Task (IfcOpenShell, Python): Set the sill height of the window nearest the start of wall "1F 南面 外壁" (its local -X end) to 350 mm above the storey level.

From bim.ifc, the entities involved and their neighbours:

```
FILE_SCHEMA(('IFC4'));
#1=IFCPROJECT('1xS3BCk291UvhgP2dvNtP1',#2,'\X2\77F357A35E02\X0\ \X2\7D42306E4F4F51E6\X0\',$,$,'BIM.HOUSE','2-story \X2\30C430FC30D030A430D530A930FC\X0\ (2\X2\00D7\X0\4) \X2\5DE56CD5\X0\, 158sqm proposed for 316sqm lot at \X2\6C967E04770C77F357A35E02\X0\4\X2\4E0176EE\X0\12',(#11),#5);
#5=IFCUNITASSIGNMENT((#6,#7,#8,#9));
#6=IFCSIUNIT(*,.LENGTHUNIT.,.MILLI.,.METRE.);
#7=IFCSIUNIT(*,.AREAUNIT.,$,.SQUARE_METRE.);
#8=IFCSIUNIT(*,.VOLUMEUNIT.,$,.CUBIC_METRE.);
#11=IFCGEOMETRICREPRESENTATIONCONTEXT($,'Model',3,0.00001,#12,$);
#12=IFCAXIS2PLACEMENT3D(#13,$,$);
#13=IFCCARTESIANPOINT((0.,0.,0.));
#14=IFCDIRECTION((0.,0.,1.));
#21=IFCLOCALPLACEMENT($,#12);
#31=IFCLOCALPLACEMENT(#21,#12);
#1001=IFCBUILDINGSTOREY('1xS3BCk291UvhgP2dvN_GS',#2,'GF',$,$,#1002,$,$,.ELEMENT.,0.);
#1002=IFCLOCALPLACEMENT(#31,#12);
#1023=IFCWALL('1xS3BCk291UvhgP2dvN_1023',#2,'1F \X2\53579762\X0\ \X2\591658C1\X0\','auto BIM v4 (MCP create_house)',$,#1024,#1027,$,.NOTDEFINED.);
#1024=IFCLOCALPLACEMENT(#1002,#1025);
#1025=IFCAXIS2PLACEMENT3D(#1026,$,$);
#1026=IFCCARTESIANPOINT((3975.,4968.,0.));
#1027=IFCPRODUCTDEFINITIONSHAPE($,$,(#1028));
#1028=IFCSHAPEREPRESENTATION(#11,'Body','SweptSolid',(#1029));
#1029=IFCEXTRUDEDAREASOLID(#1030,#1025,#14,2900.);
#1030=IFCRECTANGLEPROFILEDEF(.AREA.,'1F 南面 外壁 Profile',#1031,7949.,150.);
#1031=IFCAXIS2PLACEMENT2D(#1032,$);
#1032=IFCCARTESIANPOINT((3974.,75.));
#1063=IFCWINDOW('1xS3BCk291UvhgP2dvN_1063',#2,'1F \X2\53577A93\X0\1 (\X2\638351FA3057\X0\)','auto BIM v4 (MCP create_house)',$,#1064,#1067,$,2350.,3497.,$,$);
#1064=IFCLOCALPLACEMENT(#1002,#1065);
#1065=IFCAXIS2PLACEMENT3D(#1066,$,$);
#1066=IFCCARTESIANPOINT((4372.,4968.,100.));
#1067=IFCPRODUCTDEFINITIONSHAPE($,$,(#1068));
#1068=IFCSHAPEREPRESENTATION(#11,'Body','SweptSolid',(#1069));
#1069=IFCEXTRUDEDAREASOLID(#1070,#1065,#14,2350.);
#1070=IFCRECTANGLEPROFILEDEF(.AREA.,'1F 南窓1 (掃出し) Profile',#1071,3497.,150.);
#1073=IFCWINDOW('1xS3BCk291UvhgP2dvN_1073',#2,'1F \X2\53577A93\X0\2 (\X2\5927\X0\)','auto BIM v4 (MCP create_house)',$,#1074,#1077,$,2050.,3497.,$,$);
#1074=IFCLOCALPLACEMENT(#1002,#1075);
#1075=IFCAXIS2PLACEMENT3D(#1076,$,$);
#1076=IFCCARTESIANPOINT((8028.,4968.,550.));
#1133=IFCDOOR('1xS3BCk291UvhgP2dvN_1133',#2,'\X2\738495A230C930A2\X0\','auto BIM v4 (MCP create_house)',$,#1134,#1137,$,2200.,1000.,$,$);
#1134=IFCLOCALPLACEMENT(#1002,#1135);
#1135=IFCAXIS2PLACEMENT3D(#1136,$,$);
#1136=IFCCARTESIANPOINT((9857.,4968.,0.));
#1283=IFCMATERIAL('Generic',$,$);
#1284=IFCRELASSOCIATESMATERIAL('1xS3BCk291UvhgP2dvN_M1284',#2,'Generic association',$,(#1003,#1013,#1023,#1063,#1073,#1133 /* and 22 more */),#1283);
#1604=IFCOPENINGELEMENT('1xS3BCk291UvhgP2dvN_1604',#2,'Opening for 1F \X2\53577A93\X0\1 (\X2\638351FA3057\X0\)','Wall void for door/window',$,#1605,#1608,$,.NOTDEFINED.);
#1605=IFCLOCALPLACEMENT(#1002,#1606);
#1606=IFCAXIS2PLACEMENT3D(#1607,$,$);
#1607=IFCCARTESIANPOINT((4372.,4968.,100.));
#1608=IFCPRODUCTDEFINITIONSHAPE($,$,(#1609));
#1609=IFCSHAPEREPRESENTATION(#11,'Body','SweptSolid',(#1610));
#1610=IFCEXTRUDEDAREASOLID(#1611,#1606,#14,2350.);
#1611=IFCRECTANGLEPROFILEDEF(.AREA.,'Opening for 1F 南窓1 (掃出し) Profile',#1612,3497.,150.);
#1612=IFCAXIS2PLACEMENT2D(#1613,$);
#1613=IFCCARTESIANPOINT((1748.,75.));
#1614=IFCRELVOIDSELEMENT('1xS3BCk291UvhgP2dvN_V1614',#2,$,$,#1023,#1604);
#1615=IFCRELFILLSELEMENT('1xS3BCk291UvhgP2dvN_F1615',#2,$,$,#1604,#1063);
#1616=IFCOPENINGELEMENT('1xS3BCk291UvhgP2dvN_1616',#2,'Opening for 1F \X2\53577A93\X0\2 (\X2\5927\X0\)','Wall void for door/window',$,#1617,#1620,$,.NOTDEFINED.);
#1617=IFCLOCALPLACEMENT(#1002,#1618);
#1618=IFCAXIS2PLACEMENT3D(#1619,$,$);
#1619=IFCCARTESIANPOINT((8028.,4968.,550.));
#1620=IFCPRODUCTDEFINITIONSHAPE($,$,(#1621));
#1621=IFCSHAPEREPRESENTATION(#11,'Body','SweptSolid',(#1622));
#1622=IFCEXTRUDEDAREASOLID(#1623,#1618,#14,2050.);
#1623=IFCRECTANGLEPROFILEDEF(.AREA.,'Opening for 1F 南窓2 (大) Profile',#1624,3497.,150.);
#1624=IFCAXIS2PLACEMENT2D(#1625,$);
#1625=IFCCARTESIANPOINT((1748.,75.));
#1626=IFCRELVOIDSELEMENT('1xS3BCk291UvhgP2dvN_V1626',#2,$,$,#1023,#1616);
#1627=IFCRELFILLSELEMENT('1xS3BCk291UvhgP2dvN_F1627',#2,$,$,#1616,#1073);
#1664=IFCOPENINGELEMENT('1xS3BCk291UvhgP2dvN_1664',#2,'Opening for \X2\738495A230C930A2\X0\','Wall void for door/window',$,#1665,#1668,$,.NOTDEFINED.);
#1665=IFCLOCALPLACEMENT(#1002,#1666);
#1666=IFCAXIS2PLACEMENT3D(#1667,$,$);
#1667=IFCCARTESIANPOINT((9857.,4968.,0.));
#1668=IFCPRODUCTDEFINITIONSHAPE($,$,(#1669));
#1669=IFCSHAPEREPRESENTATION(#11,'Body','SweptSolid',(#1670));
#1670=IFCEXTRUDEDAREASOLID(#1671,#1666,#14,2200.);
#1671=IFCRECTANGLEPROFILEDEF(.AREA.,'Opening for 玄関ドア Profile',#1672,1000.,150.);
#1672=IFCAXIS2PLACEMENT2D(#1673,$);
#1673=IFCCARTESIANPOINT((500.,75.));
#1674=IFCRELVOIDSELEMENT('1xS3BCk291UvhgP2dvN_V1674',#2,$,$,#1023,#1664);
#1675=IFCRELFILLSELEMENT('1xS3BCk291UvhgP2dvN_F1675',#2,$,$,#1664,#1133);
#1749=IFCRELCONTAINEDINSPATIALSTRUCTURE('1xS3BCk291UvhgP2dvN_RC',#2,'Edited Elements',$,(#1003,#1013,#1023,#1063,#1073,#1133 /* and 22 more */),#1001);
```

```python
import numpy as np
import ifcopenshell
import ifcopenshell.api.geometry
import ifcopenshell.geom
import ifcopenshell.util.element
import ifcopenshell.util.placement
import ifcopenshell.util.shape
import ifcopenshell.util.unit

model = ifcopenshell.open("bim.ifc")
unit_scale = ifcopenshell.util.unit.calculate_unit_scale(model)

window = model.by_id(1063)
opening = window.FillsVoids[0].RelatingOpeningElement
storey = ifcopenshell.util.element.get_container(window, ifc_class="IfcBuildingStorey")
level = ifcopenshell.util.placement.get_local_placement(storey.ObjectPlacement)[2, 3]

# The opening's origin need not be at the sill, so measure its lowest point.
shape = ifcopenshell.geom.create_shape(ifcopenshell.geom.settings(), opening)
bottom = ifcopenshell.util.shape.get_shape_bottom_elevation(shape, shape.geometry) / unit_scale
dz = level + 0.35 / unit_scale - bottom

shift = np.array([0.0, 0.0, dz])
# The window is not placed relative to its opening, so move both.
for product in (opening, window):
    matrix = ifcopenshell.util.placement.get_local_placement(product.ObjectPlacement)
    matrix[:3, 3] += shift
    ifcopenshell.api.geometry.edit_object_placement(model, product=product, matrix=matrix, is_si=False)

print(f"moved by {dz * unit_scale:+.3f} m")

model.write("bim_rev.ifc")
```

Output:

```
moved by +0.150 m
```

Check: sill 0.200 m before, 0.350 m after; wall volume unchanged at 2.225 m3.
